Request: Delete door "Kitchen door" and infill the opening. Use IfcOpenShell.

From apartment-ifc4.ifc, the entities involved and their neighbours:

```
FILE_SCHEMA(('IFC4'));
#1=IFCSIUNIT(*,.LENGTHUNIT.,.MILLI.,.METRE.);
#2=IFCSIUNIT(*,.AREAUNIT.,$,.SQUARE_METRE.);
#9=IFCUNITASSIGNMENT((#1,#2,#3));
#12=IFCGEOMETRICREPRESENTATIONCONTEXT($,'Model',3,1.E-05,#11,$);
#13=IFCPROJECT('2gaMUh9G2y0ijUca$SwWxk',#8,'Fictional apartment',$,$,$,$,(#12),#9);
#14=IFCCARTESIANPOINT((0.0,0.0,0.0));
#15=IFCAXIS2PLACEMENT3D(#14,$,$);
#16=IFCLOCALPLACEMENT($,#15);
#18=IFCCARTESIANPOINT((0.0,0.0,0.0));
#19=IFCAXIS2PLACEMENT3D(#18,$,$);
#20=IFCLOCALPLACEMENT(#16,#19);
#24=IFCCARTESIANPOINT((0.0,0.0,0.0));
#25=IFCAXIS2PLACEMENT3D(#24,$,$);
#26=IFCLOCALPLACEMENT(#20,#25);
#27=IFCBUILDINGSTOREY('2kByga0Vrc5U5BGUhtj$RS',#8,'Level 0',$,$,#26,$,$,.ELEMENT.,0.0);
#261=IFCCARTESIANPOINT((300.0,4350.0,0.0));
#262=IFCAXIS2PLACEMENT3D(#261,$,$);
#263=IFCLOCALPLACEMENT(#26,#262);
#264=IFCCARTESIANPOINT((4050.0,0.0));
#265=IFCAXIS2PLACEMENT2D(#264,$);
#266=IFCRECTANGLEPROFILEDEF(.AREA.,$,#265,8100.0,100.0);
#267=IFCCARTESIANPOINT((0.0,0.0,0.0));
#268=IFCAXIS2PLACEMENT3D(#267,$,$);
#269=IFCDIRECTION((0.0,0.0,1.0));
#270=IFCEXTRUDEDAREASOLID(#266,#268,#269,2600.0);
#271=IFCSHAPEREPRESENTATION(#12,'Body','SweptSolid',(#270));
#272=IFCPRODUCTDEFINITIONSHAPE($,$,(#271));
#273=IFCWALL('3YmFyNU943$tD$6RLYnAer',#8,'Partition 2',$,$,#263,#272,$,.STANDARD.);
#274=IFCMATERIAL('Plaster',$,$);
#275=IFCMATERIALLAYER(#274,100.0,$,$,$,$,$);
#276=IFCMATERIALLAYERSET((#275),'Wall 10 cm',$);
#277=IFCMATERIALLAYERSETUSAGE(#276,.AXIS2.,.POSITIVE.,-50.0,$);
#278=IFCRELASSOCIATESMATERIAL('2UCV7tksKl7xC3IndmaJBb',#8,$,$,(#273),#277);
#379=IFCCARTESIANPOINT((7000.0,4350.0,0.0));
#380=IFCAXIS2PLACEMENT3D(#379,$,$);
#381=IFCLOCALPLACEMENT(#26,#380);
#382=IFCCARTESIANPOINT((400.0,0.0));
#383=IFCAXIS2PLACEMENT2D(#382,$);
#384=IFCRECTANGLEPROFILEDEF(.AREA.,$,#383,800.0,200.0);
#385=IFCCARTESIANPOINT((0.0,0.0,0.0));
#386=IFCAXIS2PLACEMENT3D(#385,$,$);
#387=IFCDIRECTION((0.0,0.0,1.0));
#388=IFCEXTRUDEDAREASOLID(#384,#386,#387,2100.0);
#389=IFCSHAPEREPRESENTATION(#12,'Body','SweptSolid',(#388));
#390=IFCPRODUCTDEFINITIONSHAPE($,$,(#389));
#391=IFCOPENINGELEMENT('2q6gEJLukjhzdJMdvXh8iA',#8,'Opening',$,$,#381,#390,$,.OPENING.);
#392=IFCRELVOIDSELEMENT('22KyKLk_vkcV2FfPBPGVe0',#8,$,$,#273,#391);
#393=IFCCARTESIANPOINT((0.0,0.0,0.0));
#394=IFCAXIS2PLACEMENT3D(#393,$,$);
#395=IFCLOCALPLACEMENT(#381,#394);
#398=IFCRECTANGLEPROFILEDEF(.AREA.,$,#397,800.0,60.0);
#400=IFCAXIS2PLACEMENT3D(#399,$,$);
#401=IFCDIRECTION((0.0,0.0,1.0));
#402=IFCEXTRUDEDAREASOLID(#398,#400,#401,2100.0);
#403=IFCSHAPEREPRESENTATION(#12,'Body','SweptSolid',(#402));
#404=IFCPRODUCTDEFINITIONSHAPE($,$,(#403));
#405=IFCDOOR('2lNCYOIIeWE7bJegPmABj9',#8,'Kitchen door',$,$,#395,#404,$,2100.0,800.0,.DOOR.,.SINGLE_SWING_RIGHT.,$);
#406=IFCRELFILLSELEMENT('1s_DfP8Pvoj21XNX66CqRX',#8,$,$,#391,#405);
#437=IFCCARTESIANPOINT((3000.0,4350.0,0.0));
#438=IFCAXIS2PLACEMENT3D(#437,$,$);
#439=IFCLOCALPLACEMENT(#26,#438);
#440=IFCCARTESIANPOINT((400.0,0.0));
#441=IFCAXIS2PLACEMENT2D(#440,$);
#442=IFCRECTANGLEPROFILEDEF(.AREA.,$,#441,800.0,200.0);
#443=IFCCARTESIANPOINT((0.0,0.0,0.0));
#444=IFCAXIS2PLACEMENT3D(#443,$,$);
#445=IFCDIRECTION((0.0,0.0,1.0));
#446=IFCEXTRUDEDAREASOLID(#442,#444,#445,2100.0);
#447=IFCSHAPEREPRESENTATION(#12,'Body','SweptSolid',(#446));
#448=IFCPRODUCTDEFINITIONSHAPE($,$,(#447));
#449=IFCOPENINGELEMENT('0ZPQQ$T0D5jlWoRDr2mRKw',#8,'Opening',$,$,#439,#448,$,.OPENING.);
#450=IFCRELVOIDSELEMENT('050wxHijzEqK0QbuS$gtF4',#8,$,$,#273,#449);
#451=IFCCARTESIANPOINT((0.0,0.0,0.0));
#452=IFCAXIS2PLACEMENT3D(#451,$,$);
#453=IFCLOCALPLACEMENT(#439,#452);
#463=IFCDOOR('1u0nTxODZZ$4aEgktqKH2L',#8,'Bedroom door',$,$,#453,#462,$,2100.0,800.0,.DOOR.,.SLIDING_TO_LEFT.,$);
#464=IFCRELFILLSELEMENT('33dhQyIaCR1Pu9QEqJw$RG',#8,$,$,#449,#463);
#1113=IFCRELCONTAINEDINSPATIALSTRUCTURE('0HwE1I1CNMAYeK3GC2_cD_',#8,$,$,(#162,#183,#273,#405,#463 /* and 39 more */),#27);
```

```python
import ifcopenshell
import ifcopenshell.api.feature
import ifcopenshell.api.root
import ifcopenshell.geom
import ifcopenshell.util.shape

model = ifcopenshell.open("apartment-ifc4.ifc")
settings = ifcopenshell.geom.settings()


def volume(element):
    """Net volume in cubic metres, openings subtracted."""
    shape = ifcopenshell.geom.create_shape(settings, element)
    return ifcopenshell.util.shape.get_volume(shape.geometry)


door = model.by_guid("2lNCYOIIeWE7bJegPmABj9")
opening = door.FillsVoids[0].RelatingOpeningElement
wall = opening.VoidsElements[0].RelatingBuildingElement
before = volume(wall)

ifcopenshell.api.root.remove_product(model, product=door)
ifcopenshell.api.feature.remove_feature(model, feature=opening)

after = volume(wall)

print(f"wall volume {before:.3f} -> {after:.3f} m3")

model.write("apartment-ifc4_v2.ifc")
```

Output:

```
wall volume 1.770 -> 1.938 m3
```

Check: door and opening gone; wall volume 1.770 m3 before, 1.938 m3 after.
